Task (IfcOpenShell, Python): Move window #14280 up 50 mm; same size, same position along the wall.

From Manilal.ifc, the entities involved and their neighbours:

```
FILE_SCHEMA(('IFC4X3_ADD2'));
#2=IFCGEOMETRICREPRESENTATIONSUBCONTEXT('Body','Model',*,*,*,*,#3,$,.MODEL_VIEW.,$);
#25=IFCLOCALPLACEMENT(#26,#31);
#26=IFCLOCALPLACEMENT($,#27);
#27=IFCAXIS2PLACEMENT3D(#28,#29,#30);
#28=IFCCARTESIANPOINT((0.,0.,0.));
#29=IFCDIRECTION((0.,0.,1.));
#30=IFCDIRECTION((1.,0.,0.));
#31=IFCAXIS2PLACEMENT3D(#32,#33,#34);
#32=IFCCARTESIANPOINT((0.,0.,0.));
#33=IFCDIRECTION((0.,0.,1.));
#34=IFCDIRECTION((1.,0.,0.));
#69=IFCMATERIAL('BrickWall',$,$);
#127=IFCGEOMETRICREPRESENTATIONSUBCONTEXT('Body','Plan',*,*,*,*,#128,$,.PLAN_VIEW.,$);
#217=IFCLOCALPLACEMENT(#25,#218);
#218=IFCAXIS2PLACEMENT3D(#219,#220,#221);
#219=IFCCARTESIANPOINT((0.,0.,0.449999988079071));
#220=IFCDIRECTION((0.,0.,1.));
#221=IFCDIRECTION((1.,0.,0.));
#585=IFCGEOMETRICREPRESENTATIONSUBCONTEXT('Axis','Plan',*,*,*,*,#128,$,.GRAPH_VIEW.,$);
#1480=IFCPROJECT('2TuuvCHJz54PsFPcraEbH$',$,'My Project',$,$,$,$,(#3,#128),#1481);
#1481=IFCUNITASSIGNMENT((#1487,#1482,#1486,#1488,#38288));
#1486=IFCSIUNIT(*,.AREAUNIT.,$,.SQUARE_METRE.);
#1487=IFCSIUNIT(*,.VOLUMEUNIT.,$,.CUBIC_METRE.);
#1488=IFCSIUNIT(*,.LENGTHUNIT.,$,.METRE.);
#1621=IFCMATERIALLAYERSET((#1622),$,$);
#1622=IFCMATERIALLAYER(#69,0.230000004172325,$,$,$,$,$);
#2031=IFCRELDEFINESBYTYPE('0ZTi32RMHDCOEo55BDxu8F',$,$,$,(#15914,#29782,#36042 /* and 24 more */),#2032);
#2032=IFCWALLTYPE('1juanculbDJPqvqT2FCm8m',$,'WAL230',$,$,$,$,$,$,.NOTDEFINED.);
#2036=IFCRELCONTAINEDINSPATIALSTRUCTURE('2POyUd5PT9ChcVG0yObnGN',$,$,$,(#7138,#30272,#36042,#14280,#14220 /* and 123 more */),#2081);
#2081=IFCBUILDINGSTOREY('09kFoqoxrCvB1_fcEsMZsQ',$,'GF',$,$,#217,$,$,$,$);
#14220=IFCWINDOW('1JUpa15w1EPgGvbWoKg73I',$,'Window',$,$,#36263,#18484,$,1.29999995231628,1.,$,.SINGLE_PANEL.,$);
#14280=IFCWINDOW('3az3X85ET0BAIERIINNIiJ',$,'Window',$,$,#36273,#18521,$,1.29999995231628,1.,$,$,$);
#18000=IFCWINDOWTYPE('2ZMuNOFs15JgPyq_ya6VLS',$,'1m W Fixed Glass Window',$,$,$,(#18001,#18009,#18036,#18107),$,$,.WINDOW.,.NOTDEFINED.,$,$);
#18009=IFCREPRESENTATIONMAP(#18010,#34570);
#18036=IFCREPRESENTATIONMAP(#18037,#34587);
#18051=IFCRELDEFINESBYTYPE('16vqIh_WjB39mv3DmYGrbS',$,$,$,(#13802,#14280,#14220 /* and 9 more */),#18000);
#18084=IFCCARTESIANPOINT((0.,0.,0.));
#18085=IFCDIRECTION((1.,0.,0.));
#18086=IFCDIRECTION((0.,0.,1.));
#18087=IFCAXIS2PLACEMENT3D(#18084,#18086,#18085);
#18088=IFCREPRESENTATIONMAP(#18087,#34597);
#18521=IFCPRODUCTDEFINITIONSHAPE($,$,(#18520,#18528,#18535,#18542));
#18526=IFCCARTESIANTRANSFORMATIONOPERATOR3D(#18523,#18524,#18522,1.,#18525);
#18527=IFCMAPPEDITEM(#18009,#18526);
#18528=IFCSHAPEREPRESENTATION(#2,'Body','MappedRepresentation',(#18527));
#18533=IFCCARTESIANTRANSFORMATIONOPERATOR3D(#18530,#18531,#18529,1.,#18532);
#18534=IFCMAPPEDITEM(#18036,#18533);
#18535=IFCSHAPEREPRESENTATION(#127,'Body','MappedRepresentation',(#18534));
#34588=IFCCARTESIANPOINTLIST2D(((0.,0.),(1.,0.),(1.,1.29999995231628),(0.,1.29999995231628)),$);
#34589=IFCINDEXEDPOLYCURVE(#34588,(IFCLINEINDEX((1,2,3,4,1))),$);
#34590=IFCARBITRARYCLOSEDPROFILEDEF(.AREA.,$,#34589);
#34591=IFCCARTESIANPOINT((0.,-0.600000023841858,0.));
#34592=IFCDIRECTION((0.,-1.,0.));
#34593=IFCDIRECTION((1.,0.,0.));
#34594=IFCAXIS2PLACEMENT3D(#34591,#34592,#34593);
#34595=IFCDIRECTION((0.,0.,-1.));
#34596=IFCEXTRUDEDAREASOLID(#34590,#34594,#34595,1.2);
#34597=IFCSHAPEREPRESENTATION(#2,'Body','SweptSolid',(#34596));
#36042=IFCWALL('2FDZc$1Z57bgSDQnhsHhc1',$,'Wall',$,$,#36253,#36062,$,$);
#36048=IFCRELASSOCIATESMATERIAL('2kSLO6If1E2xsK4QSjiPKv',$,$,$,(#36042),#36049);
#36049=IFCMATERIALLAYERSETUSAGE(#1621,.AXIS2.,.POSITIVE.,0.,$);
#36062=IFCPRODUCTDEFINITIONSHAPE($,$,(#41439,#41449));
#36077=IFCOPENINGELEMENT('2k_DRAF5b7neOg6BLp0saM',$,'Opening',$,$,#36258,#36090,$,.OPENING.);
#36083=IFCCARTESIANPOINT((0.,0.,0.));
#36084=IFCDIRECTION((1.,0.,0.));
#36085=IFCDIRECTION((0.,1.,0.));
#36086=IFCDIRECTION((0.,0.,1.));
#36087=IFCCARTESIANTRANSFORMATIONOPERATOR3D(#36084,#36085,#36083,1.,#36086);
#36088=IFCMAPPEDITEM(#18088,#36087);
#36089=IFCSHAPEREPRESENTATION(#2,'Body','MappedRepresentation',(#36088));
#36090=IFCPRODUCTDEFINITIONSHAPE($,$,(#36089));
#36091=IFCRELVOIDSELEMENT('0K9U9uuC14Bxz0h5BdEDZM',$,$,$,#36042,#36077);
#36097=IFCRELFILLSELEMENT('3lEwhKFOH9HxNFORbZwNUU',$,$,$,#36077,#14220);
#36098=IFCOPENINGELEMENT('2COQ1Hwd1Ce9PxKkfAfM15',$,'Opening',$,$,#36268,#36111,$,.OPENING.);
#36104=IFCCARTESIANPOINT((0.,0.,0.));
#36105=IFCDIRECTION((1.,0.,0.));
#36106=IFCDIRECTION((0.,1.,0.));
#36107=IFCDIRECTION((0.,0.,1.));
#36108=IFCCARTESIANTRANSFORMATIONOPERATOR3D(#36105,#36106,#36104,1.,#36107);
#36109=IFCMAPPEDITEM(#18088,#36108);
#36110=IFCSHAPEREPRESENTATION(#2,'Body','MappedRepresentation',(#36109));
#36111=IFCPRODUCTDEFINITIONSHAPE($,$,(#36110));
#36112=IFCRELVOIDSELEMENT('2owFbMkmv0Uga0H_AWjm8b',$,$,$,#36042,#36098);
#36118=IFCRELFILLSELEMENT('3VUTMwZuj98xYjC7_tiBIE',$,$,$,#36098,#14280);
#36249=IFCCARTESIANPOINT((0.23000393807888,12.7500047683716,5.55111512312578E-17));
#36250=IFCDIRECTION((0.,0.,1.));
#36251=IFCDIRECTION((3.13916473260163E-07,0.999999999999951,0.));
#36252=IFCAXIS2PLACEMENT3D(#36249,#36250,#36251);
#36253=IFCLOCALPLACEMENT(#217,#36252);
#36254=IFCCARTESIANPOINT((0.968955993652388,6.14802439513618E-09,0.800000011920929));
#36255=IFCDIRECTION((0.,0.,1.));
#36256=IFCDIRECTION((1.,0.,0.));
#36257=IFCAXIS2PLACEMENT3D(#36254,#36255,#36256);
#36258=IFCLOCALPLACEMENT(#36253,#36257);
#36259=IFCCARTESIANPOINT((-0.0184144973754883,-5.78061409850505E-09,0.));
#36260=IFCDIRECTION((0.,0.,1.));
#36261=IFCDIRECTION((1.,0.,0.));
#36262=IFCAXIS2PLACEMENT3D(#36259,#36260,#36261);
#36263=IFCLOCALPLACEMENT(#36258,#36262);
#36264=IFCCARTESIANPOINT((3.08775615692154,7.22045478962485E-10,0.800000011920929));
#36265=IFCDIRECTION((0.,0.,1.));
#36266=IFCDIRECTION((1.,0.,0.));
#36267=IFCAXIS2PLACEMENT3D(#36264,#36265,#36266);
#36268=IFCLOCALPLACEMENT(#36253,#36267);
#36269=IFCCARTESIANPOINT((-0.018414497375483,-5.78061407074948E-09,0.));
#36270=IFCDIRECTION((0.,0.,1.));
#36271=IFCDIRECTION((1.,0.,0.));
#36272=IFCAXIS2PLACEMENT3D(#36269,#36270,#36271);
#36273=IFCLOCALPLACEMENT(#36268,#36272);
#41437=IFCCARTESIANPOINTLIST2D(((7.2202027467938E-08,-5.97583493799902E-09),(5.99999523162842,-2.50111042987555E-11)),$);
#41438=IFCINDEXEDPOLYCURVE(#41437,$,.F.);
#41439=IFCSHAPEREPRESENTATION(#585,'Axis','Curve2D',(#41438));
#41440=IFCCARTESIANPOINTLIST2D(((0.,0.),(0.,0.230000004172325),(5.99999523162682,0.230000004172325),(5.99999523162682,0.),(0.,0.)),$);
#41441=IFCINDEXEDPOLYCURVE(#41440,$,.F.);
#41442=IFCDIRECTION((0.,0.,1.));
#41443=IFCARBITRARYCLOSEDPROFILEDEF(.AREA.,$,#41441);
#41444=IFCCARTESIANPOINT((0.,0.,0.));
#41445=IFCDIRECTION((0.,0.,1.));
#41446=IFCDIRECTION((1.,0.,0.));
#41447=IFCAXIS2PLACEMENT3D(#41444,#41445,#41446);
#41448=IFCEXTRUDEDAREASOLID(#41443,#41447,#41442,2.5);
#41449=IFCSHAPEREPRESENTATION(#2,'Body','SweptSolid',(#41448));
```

```python
import numpy as np
import ifcopenshell
import ifcopenshell.api.geometry
import ifcopenshell.util.placement
import ifcopenshell.util.unit

model = ifcopenshell.open("Manilal.ifc")
unit_scale = ifcopenshell.util.unit.calculate_unit_scale(model)

window = model.by_guid("3az3X85ET0BAIERIINNIiJ")
opening = window.FillsVoids[0].RelatingOpeningElement
dz = 0.05

shift = np.array([0.0, 0.0, dz])
# The window is placed relative to its opening, so it follows when the opening moves.
matrix = ifcopenshell.util.placement.get_local_placement(opening.ObjectPlacement)
matrix[:3, 3] += shift
ifcopenshell.api.geometry.edit_object_placement(
    model, product=opening, matrix=matrix, is_si=False, should_transform_children=True
)

print(f"moved by {dz * unit_scale:+.3f} m")

model.write("Manilal_updated.ifc")
```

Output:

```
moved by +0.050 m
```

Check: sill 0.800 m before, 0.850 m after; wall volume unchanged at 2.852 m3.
